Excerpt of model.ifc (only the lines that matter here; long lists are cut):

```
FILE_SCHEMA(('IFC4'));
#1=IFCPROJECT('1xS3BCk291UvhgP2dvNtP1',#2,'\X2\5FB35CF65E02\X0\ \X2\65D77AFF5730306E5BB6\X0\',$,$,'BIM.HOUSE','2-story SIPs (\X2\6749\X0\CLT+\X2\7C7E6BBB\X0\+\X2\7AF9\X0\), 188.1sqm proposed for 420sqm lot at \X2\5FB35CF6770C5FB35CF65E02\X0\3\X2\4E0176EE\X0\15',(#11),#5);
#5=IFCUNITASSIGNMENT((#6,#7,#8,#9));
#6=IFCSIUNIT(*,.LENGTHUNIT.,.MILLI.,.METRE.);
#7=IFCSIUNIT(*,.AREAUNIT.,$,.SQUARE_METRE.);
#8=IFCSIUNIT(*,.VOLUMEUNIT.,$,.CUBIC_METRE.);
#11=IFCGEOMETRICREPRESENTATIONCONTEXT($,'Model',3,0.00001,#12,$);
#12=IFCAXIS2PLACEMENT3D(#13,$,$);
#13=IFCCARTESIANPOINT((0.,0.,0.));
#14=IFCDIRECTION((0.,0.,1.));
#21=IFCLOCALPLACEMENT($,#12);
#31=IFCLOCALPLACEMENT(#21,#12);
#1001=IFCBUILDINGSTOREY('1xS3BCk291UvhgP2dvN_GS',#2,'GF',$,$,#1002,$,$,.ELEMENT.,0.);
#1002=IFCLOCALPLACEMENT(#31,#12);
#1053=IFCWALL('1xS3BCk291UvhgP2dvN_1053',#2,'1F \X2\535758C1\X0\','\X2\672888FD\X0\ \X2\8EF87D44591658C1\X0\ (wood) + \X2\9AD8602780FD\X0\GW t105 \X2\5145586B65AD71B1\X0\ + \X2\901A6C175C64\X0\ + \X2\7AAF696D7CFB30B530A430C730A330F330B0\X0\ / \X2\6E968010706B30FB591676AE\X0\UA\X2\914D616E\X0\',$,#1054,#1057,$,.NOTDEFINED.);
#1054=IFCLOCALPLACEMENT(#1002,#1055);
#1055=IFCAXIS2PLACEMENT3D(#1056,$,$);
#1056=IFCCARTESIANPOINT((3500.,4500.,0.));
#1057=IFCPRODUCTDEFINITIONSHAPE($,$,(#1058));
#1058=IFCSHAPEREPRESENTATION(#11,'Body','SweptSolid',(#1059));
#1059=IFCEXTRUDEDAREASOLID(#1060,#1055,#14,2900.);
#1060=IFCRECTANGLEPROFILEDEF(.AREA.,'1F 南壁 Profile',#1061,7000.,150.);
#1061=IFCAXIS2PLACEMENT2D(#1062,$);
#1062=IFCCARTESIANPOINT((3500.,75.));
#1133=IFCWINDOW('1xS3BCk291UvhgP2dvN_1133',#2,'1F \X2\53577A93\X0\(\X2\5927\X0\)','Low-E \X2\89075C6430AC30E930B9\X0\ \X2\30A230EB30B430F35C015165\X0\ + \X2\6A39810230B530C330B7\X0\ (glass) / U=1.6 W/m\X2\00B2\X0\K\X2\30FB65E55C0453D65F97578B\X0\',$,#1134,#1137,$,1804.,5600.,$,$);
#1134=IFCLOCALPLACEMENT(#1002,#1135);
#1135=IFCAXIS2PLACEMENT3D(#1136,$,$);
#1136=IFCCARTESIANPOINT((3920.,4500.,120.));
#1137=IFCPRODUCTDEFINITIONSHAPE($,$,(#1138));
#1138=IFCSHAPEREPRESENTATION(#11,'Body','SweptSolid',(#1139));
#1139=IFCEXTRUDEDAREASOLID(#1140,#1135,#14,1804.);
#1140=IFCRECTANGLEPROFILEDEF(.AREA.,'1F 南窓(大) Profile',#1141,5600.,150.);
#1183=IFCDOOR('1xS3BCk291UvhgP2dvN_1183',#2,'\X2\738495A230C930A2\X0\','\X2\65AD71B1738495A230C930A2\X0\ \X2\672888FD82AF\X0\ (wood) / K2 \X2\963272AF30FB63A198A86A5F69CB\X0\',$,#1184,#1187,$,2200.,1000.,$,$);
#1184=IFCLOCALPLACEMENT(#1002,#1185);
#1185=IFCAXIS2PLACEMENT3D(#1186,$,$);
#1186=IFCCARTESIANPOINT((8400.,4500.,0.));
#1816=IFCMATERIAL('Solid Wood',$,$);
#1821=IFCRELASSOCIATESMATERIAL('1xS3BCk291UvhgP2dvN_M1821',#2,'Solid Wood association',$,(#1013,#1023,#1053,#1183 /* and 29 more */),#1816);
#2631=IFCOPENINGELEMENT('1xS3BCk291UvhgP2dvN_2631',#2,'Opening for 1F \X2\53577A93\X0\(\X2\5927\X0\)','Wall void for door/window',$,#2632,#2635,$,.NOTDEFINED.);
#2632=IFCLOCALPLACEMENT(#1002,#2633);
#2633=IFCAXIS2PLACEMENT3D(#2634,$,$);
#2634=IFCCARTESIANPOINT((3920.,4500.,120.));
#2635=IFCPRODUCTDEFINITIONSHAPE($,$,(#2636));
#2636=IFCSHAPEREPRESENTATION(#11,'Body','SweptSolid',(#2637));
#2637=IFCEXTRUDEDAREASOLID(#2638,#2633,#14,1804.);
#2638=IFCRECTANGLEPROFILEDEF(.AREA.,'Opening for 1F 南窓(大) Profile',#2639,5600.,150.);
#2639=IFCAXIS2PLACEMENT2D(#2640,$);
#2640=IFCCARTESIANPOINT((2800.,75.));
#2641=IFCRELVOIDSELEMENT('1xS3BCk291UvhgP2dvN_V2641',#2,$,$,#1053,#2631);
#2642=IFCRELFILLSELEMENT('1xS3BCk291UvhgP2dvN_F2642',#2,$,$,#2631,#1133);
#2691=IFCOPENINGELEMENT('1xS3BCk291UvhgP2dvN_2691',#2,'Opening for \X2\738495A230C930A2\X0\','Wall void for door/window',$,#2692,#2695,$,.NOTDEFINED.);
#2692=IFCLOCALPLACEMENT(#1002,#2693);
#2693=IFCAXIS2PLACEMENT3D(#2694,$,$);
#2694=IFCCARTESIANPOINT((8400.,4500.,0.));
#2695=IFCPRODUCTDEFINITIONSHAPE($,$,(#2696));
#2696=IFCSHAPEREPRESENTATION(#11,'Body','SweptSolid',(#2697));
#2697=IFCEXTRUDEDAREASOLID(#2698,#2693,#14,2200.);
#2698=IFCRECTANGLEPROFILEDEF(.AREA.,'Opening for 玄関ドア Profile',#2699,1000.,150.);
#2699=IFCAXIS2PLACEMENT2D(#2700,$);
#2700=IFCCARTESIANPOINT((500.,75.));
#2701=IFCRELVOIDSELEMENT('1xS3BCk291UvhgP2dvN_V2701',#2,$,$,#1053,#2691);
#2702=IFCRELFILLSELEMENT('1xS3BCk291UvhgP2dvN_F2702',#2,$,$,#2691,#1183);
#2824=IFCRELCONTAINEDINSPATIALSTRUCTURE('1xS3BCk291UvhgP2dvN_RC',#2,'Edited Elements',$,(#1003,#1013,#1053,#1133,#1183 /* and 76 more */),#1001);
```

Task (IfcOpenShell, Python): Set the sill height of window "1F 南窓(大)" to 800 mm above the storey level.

```python
import numpy as np
import ifcopenshell
import ifcopenshell.api.geometry
import ifcopenshell.geom
import ifcopenshell.util.element
import ifcopenshell.util.placement
import ifcopenshell.util.shape
import ifcopenshell.util.unit

model = ifcopenshell.open("model.ifc")
unit_scale = ifcopenshell.util.unit.calculate_unit_scale(model)

window = model.by_id(1133)
opening = window.FillsVoids[0].RelatingOpeningElement
storey = ifcopenshell.util.element.get_container(window, ifc_class="IfcBuildingStorey")
level = ifcopenshell.util.placement.get_local_placement(storey.ObjectPlacement)[2, 3]

# The opening's origin need not be at the sill, so measure its lowest point.
shape = ifcopenshell.geom.create_shape(ifcopenshell.geom.settings(), opening)
bottom = ifcopenshell.util.shape.get_shape_bottom_elevation(shape, shape.geometry) / unit_scale
dz = level + 0.8 / unit_scale - bottom

shift = np.array([0.0, 0.0, dz])
# The window is not placed relative to its opening, so move both.
for product in (opening, window):
    matrix = ifcopenshell.util.placement.get_local_placement(product.ObjectPlacement)
    matrix[:3, 3] += shift
    ifcopenshell.api.geometry.edit_object_placement(model, product=product, matrix=matrix, is_si=False)

print(f"moved by {dz * unit_scale:+.3f} m")

model.write("model_rev.ifc")
```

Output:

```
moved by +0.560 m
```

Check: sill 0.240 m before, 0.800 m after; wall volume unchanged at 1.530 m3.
